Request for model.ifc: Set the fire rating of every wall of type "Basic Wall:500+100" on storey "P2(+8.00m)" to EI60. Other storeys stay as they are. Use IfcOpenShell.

First a look at what the model holds.

```python
import ifcopenshell
import ifcopenshell.util.element

model = ifcopenshell.open("model.ifc")
print(model.schema)
storey = next(s for s in model.by_type("IfcBuildingStorey") if s.Name == "P2(+8.00m)")
walls = [e for e in ifcopenshell.util.element.get_decomposition(storey) if e.is_a("IfcWall")]
seen = {}
for e in walls:
    element_type = ifcopenshell.util.element.get_type(e)
    key = (element_type.Name if element_type != e and element_type else None, ifcopenshell.util.element.get_pset(e, "Pset_WallCommon", "FireRating"))
    seen[key] = seen.get(key, 0) + 1
for (name, value), count in sorted(seen.items(), key=str):
    print(count, "x", name, "|", value)
```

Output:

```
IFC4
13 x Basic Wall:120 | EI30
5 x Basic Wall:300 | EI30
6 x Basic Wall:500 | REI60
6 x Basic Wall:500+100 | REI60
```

```python
import ifcopenshell
import ifcopenshell.api.pset
import ifcopenshell.util.element

model = ifcopenshell.open("model.ifc")

storey = next(s for s in model.by_type("IfcBuildingStorey") if s.Name == "P2(+8.00m)")
walls = [e for e in ifcopenshell.util.element.get_decomposition(storey) if e.is_a("IfcWall")]

count = 0
for e in walls:
    element_type = ifcopenshell.util.element.get_type(e)
    if element_type in (None, e) or element_type.Name != "Basic Wall:500+100":
        continue
    # add_pset returns the element's existing set when there is one.
    pset = ifcopenshell.api.pset.add_pset(model, product=e, name="Pset_WallCommon")
    ifcopenshell.api.pset.edit_pset(model, pset=pset, properties={"FireRating": "EI60"})
    count += 1

print(count, "walls updated")

model.write("model_updated.ifc")
```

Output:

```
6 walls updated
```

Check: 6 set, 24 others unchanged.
